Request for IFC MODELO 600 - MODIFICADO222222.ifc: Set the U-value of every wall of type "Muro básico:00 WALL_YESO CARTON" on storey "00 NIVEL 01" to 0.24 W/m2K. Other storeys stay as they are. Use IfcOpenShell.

First a look at what the model holds.

```python
import ifcopenshell
import ifcopenshell.util.element

model = ifcopenshell.open("IFC MODELO 600 - MODIFICADO222222.ifc")
print(model.schema)
storey = next(s for s in model.by_type("IfcBuildingStorey") if s.Name == "00 NIVEL 01")
walls = [e for e in ifcopenshell.util.element.get_decomposition(storey) if e.is_a("IfcWall")]
seen = {}
for e in walls:
    element_type = ifcopenshell.util.element.get_type(e)
    key = (element_type.Name if element_type != e and element_type else None, ifcopenshell.util.element.get_pset(e, "Pset_WallCommon", "ThermalTransmittance"))
    seen[key] = seen.get(key, 0) + 1
for (name, value), count in sorted(seen.items(), key=str):
    print(count, "x", name, "|", value)
```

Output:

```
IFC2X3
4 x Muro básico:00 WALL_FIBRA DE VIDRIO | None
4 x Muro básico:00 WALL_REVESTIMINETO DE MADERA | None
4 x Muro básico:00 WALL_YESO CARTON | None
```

```python
import ifcopenshell
import ifcopenshell.api.pset
import ifcopenshell.util.element

model = ifcopenshell.open("IFC MODELO 600 - MODIFICADO222222.ifc")

storey = next(s for s in model.by_type("IfcBuildingStorey") if s.Name == "00 NIVEL 01")
walls = [e for e in ifcopenshell.util.element.get_decomposition(storey) if e.is_a("IfcWall")]

count = 0
for e in walls:
    element_type = ifcopenshell.util.element.get_type(e)
    if element_type in (None, e) or element_type.Name != "Muro básico:00 WALL_YESO CARTON":
        continue
    # add_pset returns the element's existing set when there is one.
    pset = ifcopenshell.api.pset.add_pset(model, product=e, name="Pset_WallCommon")
    ifcopenshell.api.pset.edit_pset(model, pset=pset, properties={"ThermalTransmittance": 0.24})
    count += 1

print(count, "walls updated")

model.write("IFC MODELO 600 - MODIFICADO222222_v2.ifc")
```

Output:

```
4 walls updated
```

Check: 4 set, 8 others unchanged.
